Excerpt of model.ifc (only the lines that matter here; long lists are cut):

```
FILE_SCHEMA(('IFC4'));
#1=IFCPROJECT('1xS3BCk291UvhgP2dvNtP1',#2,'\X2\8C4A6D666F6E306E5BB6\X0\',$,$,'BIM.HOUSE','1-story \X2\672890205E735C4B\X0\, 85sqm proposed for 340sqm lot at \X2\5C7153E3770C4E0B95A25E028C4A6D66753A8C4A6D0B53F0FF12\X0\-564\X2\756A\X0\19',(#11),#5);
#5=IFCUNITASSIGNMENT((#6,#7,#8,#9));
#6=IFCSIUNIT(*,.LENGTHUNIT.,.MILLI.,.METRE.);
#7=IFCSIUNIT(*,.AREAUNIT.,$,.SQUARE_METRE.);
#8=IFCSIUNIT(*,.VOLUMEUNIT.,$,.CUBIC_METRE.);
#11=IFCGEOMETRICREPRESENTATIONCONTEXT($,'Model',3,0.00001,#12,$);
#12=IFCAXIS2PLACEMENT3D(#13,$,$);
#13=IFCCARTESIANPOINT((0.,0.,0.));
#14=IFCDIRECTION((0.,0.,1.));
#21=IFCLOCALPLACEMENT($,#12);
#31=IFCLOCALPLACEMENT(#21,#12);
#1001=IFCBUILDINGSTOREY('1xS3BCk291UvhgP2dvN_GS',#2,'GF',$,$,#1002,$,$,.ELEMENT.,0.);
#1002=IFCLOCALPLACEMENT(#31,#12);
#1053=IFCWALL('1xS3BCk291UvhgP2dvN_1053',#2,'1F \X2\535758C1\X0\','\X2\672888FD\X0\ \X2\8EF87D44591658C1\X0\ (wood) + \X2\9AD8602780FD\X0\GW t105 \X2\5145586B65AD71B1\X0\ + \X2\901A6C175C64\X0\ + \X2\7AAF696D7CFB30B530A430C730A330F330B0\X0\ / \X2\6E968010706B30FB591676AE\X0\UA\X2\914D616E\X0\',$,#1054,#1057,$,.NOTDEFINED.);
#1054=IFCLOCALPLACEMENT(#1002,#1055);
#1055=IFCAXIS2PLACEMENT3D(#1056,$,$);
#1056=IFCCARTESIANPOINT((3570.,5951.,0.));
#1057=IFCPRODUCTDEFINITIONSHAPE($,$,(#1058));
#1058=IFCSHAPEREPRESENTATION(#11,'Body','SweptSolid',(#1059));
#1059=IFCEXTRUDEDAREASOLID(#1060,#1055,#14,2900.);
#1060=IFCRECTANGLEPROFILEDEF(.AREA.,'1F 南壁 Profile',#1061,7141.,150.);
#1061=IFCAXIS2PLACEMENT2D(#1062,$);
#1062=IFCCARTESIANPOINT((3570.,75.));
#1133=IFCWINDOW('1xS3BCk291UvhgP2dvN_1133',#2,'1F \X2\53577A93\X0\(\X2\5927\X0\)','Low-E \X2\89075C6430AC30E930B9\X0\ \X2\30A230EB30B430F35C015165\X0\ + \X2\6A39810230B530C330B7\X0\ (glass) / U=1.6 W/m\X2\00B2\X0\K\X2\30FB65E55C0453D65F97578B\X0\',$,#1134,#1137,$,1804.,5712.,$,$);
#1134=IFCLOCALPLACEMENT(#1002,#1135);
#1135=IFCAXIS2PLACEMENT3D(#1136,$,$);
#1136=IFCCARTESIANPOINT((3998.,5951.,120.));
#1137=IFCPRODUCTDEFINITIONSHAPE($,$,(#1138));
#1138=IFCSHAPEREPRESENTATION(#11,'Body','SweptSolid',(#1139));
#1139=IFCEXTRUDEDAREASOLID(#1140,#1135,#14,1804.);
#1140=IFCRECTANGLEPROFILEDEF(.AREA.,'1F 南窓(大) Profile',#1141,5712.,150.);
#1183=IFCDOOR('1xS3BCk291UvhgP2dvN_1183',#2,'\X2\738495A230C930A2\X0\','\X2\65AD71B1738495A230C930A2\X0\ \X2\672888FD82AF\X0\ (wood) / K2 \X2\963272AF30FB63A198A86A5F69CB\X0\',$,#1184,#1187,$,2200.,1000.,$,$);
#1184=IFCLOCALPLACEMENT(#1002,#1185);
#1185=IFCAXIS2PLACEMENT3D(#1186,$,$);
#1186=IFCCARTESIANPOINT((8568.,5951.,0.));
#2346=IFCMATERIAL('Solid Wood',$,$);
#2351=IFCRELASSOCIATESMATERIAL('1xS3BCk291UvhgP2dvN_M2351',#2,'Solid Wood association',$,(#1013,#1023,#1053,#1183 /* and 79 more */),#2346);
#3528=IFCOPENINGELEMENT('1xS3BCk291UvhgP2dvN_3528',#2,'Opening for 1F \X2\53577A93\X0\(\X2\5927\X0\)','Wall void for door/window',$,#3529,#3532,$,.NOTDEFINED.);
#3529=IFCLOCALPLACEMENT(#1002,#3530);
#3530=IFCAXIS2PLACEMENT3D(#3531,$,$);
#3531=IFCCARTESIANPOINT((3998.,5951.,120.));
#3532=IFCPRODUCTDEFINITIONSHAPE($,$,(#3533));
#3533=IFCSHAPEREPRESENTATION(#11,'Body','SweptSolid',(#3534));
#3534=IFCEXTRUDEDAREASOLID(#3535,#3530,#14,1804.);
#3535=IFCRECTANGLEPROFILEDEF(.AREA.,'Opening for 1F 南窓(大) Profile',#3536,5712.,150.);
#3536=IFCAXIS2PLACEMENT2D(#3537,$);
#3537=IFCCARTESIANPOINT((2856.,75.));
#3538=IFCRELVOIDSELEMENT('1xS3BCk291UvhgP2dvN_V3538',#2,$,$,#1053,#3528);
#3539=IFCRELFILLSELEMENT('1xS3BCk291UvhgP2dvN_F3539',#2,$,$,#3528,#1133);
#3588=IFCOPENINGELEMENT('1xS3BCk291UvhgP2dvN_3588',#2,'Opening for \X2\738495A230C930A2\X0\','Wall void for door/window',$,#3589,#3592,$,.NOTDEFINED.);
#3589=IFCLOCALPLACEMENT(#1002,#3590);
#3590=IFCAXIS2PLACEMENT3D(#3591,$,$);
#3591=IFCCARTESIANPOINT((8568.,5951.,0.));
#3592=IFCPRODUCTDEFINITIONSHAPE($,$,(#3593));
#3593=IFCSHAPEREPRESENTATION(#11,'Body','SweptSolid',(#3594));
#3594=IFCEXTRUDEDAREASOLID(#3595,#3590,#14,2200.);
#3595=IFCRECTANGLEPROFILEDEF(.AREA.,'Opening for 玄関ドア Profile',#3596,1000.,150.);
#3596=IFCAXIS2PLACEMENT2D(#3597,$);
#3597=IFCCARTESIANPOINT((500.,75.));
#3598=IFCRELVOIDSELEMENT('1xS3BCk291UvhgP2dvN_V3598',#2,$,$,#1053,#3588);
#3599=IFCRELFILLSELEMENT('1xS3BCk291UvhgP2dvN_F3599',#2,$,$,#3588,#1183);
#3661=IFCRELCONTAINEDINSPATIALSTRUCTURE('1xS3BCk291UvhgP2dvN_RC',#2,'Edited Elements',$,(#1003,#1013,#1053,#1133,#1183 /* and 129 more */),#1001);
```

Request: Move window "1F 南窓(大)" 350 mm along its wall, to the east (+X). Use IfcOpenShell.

```python
import ifcopenshell
import ifcopenshell.api.geometry
import ifcopenshell.util.placement

model = ifcopenshell.open("model.ifc")

window = model.by_guid("1xS3BCk291UvhgP2dvN_1133")
opening = window.FillsVoids[0].RelatingOpeningElement
wall = opening.VoidsElements[0].RelatingBuildingElement

wall_matrix = ifcopenshell.util.placement.get_local_placement(wall.ObjectPlacement)
shift = wall_matrix[:3, 0] * 350.0
before = ifcopenshell.util.placement.get_local_placement(window.ObjectPlacement)[:3, 3].copy()

# The window is not placed relative to its opening, so move both.
for product in (opening, window):
    matrix = ifcopenshell.util.placement.get_local_placement(product.ObjectPlacement)
    matrix[:3, 3] += shift
    ifcopenshell.api.geometry.edit_object_placement(model, product=product, matrix=matrix, is_si=False)

after = ifcopenshell.util.placement.get_local_placement(window.ObjectPlacement)[:3, 3]
print("window moved by", (after - before).round(3) + 0.0)

model.write("model_updated.ifc")
```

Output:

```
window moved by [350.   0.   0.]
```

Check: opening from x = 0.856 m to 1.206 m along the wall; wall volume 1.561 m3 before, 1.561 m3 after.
